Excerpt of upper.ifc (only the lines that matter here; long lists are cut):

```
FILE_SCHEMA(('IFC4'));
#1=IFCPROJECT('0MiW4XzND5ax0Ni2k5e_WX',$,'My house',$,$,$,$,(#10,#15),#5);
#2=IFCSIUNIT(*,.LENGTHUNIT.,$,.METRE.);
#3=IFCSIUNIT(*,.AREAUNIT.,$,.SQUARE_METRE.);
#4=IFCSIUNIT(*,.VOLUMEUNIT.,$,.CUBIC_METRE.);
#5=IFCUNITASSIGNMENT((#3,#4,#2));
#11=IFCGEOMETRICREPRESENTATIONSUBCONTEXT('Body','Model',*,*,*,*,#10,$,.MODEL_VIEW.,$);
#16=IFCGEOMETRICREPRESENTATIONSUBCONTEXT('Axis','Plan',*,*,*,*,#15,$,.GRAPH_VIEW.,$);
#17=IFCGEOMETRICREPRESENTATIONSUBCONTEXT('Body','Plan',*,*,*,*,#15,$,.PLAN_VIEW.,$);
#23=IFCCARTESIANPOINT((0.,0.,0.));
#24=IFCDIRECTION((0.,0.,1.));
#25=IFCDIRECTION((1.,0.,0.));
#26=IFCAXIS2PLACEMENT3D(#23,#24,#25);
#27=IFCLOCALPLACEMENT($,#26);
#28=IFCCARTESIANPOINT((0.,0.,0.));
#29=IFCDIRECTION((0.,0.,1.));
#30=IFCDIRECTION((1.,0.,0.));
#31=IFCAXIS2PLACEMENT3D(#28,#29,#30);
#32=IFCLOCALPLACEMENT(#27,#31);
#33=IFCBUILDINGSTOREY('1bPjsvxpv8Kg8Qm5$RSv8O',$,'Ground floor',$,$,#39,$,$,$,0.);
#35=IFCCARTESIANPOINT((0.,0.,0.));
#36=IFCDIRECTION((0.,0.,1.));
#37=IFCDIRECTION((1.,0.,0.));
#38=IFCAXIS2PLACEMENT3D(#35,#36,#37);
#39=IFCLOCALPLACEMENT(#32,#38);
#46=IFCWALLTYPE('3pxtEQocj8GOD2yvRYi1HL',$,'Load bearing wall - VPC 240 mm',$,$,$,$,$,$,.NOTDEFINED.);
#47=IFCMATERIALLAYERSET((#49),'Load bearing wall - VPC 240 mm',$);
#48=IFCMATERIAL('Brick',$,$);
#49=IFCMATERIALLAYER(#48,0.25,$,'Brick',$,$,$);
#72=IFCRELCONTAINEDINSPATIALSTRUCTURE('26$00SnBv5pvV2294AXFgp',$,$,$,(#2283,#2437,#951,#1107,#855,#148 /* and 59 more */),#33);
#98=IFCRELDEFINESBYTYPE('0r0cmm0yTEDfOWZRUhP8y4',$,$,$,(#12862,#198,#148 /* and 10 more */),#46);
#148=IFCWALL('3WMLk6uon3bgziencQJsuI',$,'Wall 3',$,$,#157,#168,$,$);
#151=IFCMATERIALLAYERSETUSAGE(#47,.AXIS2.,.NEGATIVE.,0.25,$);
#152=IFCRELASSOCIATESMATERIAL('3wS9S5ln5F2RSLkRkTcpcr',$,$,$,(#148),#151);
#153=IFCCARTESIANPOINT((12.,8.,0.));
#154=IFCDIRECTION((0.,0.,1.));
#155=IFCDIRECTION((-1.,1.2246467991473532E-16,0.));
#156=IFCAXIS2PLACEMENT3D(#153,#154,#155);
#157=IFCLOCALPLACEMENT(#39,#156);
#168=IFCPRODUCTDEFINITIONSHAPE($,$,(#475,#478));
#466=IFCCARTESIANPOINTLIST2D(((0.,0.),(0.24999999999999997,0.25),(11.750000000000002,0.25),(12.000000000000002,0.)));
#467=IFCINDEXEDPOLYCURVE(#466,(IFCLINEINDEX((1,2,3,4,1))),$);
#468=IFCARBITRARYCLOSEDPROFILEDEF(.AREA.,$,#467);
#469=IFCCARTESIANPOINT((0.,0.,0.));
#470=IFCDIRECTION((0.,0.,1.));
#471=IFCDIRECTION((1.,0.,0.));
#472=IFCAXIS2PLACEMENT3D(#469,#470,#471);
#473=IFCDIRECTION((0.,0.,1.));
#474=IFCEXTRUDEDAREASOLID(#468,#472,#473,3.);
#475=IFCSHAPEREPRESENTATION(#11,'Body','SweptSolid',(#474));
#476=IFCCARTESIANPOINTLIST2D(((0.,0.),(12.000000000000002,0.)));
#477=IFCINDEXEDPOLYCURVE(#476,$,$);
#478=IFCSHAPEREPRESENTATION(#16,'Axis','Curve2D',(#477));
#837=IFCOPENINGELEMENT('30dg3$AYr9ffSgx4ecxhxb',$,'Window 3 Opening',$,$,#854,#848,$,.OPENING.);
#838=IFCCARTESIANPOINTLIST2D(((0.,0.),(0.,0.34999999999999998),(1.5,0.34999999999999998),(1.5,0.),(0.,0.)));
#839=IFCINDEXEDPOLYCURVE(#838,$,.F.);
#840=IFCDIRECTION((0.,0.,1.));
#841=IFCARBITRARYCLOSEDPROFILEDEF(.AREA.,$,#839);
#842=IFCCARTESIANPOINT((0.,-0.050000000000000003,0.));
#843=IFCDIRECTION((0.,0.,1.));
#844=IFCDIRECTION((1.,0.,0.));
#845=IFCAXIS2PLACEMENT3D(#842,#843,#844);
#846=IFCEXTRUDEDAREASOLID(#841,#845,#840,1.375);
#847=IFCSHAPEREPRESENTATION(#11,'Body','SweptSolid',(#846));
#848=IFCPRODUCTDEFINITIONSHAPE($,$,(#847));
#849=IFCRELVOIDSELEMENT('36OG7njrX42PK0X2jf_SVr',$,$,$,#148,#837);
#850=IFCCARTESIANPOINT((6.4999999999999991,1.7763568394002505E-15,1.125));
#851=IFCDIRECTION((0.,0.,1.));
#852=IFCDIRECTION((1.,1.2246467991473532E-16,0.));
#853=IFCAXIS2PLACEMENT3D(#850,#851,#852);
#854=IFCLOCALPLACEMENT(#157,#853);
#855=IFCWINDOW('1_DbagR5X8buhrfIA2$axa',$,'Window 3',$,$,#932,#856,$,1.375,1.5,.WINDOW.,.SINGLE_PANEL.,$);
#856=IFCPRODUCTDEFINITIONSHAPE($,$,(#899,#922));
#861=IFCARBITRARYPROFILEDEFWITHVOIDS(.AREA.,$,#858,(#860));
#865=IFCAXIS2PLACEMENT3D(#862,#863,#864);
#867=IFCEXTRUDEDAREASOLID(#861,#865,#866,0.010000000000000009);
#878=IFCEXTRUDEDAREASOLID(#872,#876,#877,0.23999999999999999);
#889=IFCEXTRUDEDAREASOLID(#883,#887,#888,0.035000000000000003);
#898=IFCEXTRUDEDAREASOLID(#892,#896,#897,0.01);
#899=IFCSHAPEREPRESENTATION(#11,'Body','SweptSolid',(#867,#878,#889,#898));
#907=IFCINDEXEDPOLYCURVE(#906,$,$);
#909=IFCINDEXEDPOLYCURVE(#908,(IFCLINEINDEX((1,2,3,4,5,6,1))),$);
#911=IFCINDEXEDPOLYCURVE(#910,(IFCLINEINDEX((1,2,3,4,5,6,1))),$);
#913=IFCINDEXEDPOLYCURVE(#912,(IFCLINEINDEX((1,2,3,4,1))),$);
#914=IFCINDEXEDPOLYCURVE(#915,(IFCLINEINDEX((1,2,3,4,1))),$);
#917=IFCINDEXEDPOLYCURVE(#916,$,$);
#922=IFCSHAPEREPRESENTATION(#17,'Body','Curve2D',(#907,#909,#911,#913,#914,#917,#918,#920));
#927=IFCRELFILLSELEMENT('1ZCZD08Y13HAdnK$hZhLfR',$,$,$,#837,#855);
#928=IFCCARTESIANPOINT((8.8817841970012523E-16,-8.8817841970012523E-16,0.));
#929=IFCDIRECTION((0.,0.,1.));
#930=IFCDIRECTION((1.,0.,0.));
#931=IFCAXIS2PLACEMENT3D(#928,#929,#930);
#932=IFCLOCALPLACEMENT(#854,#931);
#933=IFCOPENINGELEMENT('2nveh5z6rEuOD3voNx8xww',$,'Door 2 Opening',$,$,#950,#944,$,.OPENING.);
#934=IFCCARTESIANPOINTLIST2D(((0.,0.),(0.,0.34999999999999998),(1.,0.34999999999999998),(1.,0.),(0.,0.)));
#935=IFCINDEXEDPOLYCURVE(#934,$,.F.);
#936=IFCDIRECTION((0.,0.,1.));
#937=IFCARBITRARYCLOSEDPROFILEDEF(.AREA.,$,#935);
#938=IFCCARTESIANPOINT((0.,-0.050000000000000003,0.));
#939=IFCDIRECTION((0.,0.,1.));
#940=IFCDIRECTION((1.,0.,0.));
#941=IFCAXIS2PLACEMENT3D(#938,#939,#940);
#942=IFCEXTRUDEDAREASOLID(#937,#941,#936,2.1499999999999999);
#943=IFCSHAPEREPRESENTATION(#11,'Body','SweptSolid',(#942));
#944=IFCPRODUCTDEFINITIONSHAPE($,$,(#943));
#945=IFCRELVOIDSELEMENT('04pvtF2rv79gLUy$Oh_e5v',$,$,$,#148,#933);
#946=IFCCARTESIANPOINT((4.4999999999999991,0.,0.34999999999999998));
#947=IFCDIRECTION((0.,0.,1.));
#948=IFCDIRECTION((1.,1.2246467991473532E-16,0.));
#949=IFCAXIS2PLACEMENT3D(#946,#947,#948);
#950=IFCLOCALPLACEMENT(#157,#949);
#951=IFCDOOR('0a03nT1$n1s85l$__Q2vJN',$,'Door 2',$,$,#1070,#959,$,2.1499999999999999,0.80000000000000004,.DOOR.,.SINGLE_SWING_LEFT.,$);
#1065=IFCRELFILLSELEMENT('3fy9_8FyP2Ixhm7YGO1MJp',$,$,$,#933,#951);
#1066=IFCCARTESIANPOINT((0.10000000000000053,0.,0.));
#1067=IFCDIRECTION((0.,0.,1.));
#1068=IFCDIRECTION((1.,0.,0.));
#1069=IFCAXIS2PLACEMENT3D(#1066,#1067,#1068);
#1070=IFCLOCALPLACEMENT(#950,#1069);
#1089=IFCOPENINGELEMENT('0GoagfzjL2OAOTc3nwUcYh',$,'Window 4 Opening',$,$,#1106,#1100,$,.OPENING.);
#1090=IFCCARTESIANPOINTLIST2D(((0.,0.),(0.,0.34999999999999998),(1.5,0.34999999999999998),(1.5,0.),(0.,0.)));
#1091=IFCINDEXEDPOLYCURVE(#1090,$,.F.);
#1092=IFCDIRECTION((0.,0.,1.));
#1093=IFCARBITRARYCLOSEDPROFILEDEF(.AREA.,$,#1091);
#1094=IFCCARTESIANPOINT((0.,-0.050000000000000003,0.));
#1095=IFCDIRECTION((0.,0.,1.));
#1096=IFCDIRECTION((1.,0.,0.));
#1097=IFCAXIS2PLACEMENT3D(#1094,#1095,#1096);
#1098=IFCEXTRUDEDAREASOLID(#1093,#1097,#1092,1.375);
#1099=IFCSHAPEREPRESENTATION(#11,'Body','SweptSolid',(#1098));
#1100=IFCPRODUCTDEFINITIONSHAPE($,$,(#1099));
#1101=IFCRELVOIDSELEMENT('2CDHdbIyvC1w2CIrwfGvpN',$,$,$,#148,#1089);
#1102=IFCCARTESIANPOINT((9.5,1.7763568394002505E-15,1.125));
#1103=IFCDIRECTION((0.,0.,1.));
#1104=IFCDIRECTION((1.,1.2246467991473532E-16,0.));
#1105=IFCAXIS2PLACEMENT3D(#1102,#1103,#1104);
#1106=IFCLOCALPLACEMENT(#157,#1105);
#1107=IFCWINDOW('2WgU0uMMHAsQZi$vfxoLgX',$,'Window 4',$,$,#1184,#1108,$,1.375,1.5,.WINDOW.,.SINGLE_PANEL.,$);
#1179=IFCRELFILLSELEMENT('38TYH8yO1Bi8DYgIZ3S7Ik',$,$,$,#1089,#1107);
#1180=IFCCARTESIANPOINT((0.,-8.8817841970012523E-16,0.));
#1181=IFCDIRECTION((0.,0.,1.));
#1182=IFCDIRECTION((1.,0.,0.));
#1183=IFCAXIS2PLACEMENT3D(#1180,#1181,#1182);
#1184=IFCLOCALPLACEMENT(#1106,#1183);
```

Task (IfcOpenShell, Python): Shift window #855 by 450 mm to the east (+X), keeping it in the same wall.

```python
import ifcopenshell
import ifcopenshell.api.geometry
import ifcopenshell.util.placement
import ifcopenshell.util.unit

model = ifcopenshell.open("upper.ifc")
unit_scale = ifcopenshell.util.unit.calculate_unit_scale(model)

window = model.by_guid("1_DbagR5X8buhrfIA2$axa")
opening = window.FillsVoids[0].RelatingOpeningElement
wall = opening.VoidsElements[0].RelatingBuildingElement

wall_matrix = ifcopenshell.util.placement.get_local_placement(wall.ObjectPlacement)
shift = wall_matrix[:3, 0] * -0.45 / unit_scale
before = ifcopenshell.util.placement.get_local_placement(window.ObjectPlacement)[:3, 3].copy()

# The window is placed relative to its opening, so it follows when the opening moves.
matrix = ifcopenshell.util.placement.get_local_placement(opening.ObjectPlacement)
matrix[:3, 3] += shift
ifcopenshell.api.geometry.edit_object_placement(
    model, product=opening, matrix=matrix, is_si=False, should_transform_children=True
)

after = ifcopenshell.util.placement.get_local_placement(window.ObjectPlacement)[:3, 3]
print("window moved by", (after - before).round(3) + 0.0)

model.write("upper-out.ifc")
```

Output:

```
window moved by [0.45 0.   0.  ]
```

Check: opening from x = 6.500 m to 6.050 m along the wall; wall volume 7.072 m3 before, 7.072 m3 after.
